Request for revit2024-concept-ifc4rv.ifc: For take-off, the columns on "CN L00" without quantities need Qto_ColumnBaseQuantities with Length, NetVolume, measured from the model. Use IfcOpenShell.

First a look at what the model holds.

```python
import ifcopenshell
import ifcopenshell.util.element
import ifcopenshell.util.unit

model = ifcopenshell.open("revit2024-concept-ifc4rv.ifc")
print(model.schema)
for unit_type in ("LENGTHUNIT", "AREAUNIT", "VOLUMEUNIT"):
    print(unit_type, ifcopenshell.util.unit.calculate_unit_scale(model, unit_type))
storey = next(s for s in model.by_type("IfcBuildingStorey") if s.Name == "CN L00")
columns = [e for e in ifcopenshell.util.element.get_decomposition(storey) if e.is_a("IfcColumn")]
for e in sorted(columns, key=lambda e: e.id()):
    print(e.id(), e.is_a(), e.Name, list(ifcopenshell.util.element.get_psets(e, qtos_only=True)), sep=" | ")
```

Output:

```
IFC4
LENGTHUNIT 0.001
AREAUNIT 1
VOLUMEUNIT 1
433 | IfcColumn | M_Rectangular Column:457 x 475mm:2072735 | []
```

```python
import ifcopenshell
import ifcopenshell.api.pset
import ifcopenshell.geom
import ifcopenshell.util.element
import ifcopenshell.util.shape
import ifcopenshell.util.unit

model = ifcopenshell.open("revit2024-concept-ifc4rv.ifc")
unit_scale = ifcopenshell.util.unit.calculate_unit_scale(model)
volume_scale = ifcopenshell.util.unit.calculate_unit_scale(model, "VOLUMEUNIT")
settings = ifcopenshell.geom.settings()

storey = next(s for s in model.by_type("IfcBuildingStorey") if s.Name == "CN L00")
columns = [e for e in ifcopenshell.util.element.get_decomposition(storey) if e.is_a("IfcColumn")]

for e in sorted(columns, key=lambda e: e.id()):
    if ifcopenshell.util.element.get_psets(e, qtos_only=True, should_inherit=False):
        continue
    # Geometry comes back in metres, in the element's own axes.
    shape = ifcopenshell.geom.create_shape(settings, e)
    values = {
        "Length": ifcopenshell.util.shape.get_z(shape.geometry) / unit_scale,
        "NetVolume": ifcopenshell.util.shape.get_volume(shape.geometry) / volume_scale,
    }
    qto = ifcopenshell.api.pset.add_qto(model, product=e, name="Qto_ColumnBaseQuantities")
    ifcopenshell.api.pset.edit_qto(model, qto=qto, properties=values)
    print(e.id(), {k: round(v, 3) for k, v in values.items()})

model.write("revit2024-concept-ifc4rv_updated.ifc")
```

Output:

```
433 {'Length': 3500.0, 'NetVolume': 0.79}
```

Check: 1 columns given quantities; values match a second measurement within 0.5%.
